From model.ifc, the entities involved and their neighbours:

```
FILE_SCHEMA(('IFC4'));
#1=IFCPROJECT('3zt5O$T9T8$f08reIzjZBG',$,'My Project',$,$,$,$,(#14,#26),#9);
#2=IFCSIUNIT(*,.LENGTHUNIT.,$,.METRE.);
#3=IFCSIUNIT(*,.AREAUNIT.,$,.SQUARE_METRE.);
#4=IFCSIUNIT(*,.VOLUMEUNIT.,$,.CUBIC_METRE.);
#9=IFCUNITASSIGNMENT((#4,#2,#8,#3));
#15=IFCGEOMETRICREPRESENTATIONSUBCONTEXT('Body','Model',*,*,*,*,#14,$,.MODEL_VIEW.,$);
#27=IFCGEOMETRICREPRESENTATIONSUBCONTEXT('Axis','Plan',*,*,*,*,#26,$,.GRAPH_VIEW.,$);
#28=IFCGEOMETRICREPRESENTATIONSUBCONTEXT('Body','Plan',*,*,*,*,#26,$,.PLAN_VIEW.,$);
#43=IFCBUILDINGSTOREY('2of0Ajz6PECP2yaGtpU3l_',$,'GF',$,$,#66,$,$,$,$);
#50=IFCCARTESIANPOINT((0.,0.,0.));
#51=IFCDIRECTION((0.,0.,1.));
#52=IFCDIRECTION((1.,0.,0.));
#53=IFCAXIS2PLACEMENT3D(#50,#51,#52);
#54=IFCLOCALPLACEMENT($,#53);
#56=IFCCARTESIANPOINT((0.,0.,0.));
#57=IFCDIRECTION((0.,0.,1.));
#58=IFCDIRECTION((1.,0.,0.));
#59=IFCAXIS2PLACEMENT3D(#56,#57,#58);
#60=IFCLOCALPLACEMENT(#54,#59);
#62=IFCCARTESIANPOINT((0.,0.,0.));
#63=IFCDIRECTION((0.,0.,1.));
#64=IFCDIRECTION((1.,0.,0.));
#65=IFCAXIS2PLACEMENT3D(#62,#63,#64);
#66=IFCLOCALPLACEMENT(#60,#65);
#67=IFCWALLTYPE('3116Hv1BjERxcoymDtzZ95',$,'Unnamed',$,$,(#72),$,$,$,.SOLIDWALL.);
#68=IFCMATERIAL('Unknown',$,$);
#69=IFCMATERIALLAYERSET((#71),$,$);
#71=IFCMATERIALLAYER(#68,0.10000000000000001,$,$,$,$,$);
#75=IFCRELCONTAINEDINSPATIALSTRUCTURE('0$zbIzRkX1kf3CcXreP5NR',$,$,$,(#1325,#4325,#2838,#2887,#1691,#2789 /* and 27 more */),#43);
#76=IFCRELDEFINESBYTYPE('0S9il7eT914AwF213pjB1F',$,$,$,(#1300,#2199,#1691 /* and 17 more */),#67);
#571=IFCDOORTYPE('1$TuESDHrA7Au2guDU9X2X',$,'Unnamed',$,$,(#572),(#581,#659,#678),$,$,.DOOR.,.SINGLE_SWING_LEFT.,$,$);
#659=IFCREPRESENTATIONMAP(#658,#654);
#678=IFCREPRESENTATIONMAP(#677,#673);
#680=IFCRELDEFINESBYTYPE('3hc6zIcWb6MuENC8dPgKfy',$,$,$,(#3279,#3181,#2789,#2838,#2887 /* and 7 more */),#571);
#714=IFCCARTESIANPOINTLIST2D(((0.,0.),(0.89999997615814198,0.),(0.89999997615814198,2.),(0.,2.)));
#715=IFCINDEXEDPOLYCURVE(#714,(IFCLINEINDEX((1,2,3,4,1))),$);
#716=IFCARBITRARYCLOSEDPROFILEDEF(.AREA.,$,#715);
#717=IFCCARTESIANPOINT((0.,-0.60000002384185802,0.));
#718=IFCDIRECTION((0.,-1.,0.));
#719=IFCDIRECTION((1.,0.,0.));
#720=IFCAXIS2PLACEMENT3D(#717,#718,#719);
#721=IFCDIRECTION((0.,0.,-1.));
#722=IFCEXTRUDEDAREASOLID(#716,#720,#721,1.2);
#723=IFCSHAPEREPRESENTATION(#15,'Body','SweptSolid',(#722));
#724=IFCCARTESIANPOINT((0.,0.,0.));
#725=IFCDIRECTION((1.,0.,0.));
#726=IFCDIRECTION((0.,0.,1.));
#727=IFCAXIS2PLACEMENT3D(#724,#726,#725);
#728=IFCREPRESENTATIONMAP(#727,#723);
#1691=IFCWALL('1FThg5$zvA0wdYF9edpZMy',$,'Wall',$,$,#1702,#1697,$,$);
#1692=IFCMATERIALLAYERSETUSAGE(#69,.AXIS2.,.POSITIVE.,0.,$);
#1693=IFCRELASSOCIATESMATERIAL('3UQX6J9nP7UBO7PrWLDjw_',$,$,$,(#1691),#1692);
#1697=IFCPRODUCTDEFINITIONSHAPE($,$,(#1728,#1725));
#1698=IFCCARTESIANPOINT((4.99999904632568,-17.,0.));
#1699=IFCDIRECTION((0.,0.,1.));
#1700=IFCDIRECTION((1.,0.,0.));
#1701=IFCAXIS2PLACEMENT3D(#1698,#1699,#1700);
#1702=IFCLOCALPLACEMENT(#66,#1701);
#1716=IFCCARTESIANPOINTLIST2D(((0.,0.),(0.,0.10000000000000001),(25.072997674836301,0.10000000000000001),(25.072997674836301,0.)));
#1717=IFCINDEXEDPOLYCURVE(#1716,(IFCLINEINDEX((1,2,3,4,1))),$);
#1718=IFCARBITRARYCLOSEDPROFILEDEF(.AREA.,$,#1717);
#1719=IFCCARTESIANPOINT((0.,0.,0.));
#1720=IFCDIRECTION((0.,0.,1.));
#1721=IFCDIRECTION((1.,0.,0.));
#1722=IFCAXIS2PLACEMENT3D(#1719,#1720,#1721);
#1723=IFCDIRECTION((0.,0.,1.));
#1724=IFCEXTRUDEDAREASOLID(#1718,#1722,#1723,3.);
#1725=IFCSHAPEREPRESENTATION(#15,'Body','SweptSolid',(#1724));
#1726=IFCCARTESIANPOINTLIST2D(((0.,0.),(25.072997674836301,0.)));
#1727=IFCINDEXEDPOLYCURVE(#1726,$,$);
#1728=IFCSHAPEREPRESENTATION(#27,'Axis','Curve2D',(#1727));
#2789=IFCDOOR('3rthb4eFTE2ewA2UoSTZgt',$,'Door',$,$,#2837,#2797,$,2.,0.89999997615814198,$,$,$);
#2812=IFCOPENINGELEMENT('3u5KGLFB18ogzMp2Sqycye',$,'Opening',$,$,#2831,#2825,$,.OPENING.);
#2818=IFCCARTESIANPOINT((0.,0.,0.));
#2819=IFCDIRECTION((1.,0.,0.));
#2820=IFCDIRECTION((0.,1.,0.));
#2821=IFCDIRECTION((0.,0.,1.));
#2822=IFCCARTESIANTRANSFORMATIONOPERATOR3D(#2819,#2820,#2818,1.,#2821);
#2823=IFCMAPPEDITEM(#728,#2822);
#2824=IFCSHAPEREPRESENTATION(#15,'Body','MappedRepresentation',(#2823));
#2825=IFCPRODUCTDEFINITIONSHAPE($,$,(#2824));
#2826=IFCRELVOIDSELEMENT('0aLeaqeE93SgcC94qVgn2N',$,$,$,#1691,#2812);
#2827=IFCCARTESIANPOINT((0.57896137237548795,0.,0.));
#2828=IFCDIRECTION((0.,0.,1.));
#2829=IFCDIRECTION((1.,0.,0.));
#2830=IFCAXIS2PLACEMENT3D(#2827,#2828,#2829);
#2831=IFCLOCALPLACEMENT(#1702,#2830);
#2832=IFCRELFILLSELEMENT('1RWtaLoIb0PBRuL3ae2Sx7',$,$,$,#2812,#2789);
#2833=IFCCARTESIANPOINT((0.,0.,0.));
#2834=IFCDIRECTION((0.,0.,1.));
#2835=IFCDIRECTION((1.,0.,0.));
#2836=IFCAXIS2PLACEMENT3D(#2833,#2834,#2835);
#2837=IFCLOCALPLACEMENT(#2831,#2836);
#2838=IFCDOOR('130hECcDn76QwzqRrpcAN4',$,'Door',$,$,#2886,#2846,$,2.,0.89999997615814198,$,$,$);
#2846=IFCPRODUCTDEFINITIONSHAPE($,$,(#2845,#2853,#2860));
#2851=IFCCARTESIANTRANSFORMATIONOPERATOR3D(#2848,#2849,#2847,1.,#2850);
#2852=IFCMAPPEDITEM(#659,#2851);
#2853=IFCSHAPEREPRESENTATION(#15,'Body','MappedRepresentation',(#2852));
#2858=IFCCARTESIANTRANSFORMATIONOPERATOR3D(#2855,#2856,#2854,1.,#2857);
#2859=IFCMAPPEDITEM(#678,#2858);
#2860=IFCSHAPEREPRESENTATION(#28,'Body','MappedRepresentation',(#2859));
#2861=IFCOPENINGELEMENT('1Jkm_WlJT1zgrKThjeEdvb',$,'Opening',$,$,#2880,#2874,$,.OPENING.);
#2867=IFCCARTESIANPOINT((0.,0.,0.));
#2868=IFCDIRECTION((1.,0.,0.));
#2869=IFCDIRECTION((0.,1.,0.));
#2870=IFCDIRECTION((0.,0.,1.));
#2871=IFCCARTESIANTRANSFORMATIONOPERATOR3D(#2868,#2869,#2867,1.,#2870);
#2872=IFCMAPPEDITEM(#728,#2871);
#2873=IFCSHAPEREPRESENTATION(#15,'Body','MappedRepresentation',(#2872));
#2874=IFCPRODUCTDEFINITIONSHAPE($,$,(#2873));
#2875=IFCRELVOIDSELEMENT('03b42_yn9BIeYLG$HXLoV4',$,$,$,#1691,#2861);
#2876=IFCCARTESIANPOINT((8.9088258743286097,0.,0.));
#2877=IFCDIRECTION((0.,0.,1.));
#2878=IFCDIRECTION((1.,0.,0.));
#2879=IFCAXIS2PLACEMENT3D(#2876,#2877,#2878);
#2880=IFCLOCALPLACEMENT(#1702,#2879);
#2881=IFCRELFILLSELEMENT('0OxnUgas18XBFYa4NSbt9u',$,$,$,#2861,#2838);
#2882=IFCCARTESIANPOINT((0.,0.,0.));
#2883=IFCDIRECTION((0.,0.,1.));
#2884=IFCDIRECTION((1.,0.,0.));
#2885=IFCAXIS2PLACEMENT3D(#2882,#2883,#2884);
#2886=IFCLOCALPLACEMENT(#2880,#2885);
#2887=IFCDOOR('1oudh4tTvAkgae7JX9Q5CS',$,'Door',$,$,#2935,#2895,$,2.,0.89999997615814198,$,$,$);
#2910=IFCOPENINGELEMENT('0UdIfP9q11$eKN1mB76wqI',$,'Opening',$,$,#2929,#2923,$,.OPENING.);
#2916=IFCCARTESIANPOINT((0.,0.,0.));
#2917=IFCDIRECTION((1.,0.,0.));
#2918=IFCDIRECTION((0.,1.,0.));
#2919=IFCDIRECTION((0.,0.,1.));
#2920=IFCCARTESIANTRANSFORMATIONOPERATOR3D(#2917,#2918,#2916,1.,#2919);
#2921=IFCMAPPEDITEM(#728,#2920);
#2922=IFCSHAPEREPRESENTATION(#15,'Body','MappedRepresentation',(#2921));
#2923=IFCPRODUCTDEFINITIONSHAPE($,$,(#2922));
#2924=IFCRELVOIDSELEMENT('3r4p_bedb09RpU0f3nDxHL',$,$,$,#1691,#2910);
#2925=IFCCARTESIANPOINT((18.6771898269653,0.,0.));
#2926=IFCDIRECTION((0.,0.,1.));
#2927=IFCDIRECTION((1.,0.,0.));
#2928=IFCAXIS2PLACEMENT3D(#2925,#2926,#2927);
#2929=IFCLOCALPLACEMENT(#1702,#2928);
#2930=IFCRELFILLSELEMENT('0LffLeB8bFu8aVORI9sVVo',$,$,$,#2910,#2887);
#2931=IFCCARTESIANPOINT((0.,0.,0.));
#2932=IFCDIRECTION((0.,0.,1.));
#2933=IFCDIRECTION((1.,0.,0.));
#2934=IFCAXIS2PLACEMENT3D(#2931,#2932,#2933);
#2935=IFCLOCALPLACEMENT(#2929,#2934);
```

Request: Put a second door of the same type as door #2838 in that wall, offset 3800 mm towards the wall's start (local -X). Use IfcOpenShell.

```python
import ifcopenshell
import ifcopenshell.api.feature
import ifcopenshell.api.geometry
import ifcopenshell.api.root
import ifcopenshell.geom
import ifcopenshell.util.element
import ifcopenshell.util.placement
import ifcopenshell.util.shape
import ifcopenshell.util.unit

model = ifcopenshell.open("model.ifc")
unit_scale = ifcopenshell.util.unit.calculate_unit_scale(model)
settings = ifcopenshell.geom.settings()


def volume(element):
    """Net volume in cubic metres, openings subtracted."""
    shape = ifcopenshell.geom.create_shape(settings, element)
    return ifcopenshell.util.shape.get_volume(shape.geometry)


door = model.by_guid("130hECcDn76QwzqRrpcAN4")
opening = door.FillsVoids[0].RelatingOpeningElement
wall = opening.VoidsElements[0].RelatingBuildingElement
before = volume(wall)
shift = ifcopenshell.util.placement.get_local_placement(wall.ObjectPlacement)[:3, 0] * -3.8 / unit_scale

# copy_class copies the void relationship, type, container and properties, but no geometry.
new_opening = ifcopenshell.api.root.copy_class(model, product=opening)
new_opening.Representation = ifcopenshell.util.element.copy_deep(
    model, opening.Representation, exclude=["IfcGeometricRepresentationContext", "IfcRepresentationMap"]
)
new_door = ifcopenshell.api.root.copy_class(model, product=door)
new_door.Representation = ifcopenshell.util.element.copy_deep(
    model, door.Representation, exclude=["IfcGeometricRepresentationContext", "IfcRepresentationMap"]
)
ifcopenshell.api.feature.add_filling(model, opening=new_opening, element=new_door)

for old, new in ((opening, new_opening), (door, new_door)):
    matrix = ifcopenshell.util.placement.get_local_placement(old.ObjectPlacement)
    matrix[:3, 3] += shift
    ifcopenshell.api.geometry.edit_object_placement(model, product=new, matrix=matrix, is_si=False)

after = volume(wall)

print(f"wall volume {before:.3f} -> {after:.3f} m3")

model.write("model_rev.ifc")
```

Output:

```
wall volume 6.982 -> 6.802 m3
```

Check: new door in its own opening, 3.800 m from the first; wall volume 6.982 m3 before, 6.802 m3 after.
